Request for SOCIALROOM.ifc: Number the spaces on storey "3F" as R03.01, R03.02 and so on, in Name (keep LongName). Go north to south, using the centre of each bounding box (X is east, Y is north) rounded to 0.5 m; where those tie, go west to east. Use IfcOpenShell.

First a look at what the model holds.

```python
import ifcopenshell
import ifcopenshell.util.element
import ifcopenshell.util.placement

model = ifcopenshell.open("SOCIALROOM.ifc")
print(model.schema)
storey = next(s for s in model.by_type("IfcBuildingStorey") if s.Name == "3F")
spaces = [e for e in ifcopenshell.util.element.get_decomposition(storey) if e.is_a("IfcSpace")]
for e in sorted(spaces, key=lambda e: e.id()):
    origin = ifcopenshell.util.placement.get_local_placement(e.ObjectPlacement)[:3, 3]
    print(e.id(), e.Name, e.LongName, origin.round(2) + 0.0, sep=" | ")
```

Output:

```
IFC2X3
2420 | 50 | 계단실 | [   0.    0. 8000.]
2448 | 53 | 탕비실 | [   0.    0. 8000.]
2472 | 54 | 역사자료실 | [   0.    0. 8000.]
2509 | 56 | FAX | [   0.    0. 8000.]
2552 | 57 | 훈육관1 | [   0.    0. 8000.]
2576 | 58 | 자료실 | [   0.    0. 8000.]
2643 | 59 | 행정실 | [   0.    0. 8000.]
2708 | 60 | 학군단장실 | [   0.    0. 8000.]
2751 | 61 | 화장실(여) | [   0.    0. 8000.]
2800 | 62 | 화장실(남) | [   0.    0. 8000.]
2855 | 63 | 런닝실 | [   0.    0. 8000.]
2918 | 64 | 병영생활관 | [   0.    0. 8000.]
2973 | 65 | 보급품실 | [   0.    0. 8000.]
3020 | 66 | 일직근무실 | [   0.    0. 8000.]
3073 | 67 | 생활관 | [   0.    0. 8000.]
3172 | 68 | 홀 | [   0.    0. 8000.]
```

```python
import ifcopenshell
import ifcopenshell.geom
import ifcopenshell.util.element
import ifcopenshell.util.shape

model = ifcopenshell.open("SOCIALROOM.ifc")
settings = ifcopenshell.geom.settings()
settings.set("use-world-coords", True)


def centre(element):
    shape = ifcopenshell.geom.create_shape(settings, element)
    return ifcopenshell.util.shape.get_bbox_centroid(shape.geometry)


storey = next(s for s in model.by_type("IfcBuildingStorey") if s.Name == "3F")
spaces = [e for e in ifcopenshell.util.element.get_decomposition(storey) if e.is_a("IfcSpace")]

# Insertion points can sit at a corner or the storey origin, so sort by the geometry (in metres).
centres = {e: centre(e) for e in spaces}
spaces.sort(key=lambda e: (-round(centres[e][1] / 0.5), centres[e][0]))

for i, e in enumerate(spaces, start=1):
    number = f"R03.{i:02d}"
    e.Name = number
    print(e.id(), number)

model.write("SOCIALROOM_updated.ifc")
```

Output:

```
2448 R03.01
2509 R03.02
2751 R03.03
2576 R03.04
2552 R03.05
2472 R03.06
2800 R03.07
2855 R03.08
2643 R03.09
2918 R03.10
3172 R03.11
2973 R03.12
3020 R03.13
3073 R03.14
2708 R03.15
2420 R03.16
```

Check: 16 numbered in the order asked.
